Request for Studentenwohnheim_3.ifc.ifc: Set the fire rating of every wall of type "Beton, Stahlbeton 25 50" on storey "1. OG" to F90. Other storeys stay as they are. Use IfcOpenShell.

First a look at what the model holds.

```python
import ifcopenshell
import ifcopenshell.util.element

model = ifcopenshell.open("Studentenwohnheim_3.ifc.ifc")
print(model.schema)
storey = next(s for s in model.by_type("IfcBuildingStorey") if s.Name == "1. OG")
walls = [e for e in ifcopenshell.util.element.get_decomposition(storey) if e.is_a("IfcWall")]
seen = {}
for e in walls:
    element_type = ifcopenshell.util.element.get_type(e)
    key = (element_type.Name if element_type != e and element_type else None, ifcopenshell.util.element.get_pset(e, "Pset_WallCommon", "FireRating"))
    seen[key] = seen.get(key, 0) + 1
for (name, value), count in sorted(seen.items(), key=str):
    print(count, "x", name, "|", value)
```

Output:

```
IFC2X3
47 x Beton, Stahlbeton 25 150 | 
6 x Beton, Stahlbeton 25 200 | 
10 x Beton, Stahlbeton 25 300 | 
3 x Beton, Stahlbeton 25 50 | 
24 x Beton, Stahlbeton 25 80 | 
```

```python
import ifcopenshell
import ifcopenshell.api.pset
import ifcopenshell.util.element

model = ifcopenshell.open("Studentenwohnheim_3.ifc.ifc")

storey = next(s for s in model.by_type("IfcBuildingStorey") if s.Name == "1. OG")
walls = [e for e in ifcopenshell.util.element.get_decomposition(storey) if e.is_a("IfcWall")]

count = 0
for e in walls:
    element_type = ifcopenshell.util.element.get_type(e)
    if element_type in (None, e) or element_type.Name != "Beton, Stahlbeton 25 50":
        continue
    # add_pset returns the element's existing set when there is one.
    pset = ifcopenshell.api.pset.add_pset(model, product=e, name="Pset_WallCommon")
    ifcopenshell.api.pset.edit_pset(model, pset=pset, properties={"FireRating": "F90"})
    count += 1

print(count, "walls updated")

model.write("Studentenwohnheim_3.ifc_v2.ifc")
```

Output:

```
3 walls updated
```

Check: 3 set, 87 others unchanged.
